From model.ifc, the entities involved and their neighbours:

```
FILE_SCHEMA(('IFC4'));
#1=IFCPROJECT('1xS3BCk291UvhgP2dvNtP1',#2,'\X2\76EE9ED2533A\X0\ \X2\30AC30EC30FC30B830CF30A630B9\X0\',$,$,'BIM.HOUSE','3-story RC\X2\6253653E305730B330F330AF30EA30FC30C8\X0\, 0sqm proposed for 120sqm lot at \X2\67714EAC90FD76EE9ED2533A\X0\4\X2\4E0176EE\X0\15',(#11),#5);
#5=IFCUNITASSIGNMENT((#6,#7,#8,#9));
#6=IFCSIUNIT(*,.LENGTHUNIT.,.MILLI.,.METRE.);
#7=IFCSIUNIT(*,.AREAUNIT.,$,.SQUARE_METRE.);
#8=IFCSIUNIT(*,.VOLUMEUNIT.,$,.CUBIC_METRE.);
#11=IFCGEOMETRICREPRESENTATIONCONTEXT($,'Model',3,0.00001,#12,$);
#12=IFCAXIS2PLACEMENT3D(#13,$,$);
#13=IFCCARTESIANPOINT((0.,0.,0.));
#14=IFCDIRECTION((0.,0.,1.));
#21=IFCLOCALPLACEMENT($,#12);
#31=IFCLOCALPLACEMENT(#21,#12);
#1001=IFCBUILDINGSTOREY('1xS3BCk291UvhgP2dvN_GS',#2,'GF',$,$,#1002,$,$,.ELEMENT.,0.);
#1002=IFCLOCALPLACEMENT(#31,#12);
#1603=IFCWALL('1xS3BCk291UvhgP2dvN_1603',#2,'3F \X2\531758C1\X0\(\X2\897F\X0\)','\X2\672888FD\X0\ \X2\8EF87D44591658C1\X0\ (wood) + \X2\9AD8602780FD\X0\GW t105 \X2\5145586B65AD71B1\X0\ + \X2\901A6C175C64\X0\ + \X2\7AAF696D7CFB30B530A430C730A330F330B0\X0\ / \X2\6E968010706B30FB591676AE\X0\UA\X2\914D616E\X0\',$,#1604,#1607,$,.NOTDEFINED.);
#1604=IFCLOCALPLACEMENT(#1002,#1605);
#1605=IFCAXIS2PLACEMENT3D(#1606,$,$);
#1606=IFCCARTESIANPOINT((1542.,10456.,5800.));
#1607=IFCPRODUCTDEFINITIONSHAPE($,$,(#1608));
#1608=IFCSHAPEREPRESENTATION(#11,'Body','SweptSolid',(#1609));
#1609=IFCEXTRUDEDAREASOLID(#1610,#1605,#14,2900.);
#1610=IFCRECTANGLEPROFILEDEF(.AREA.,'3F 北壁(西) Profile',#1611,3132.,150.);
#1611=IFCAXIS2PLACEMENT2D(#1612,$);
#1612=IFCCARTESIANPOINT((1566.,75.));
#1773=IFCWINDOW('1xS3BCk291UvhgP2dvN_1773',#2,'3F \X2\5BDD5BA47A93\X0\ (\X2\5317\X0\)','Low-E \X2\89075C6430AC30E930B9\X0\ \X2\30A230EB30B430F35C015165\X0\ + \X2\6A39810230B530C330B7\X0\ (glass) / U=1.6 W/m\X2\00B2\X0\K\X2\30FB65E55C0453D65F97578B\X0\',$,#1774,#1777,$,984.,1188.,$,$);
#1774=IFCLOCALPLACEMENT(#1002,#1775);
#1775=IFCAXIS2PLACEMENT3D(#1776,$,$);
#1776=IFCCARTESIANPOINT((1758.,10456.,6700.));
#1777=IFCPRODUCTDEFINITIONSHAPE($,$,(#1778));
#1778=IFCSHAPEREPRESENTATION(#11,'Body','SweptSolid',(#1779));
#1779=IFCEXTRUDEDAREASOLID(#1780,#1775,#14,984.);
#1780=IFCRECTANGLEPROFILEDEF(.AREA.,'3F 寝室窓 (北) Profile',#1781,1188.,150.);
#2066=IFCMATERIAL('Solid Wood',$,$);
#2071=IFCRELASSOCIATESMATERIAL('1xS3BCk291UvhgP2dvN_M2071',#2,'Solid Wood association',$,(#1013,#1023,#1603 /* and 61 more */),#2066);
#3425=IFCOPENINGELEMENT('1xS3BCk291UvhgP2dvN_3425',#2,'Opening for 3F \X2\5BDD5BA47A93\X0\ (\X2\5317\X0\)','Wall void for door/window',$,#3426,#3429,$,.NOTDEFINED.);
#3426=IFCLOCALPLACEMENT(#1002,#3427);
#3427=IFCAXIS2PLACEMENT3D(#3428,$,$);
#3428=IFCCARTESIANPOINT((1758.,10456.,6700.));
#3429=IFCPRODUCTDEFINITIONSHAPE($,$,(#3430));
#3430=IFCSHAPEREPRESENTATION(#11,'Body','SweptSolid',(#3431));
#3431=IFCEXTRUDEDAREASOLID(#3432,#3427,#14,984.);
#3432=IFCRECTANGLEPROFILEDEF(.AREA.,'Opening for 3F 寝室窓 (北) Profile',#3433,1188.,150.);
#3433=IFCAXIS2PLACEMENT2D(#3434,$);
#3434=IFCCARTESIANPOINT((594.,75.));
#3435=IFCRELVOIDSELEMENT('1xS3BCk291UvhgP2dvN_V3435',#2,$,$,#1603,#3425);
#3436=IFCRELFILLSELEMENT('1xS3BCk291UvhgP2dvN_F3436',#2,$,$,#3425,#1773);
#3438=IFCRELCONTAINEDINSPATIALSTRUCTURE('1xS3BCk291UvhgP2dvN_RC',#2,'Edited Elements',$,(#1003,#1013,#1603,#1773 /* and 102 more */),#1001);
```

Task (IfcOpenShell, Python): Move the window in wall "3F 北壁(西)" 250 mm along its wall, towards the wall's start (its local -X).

```python
import ifcopenshell
import ifcopenshell.api.geometry
import ifcopenshell.util.placement

model = ifcopenshell.open("model.ifc")

window = model.by_guid("1xS3BCk291UvhgP2dvN_1773")
opening = window.FillsVoids[0].RelatingOpeningElement
wall = opening.VoidsElements[0].RelatingBuildingElement

wall_matrix = ifcopenshell.util.placement.get_local_placement(wall.ObjectPlacement)
shift = wall_matrix[:3, 0] * -250.0
before = ifcopenshell.util.placement.get_local_placement(window.ObjectPlacement)[:3, 3].copy()

# The window is not placed relative to its opening, so move both.
for product in (opening, window):
    matrix = ifcopenshell.util.placement.get_local_placement(product.ObjectPlacement)
    matrix[:3, 3] += shift
    ifcopenshell.api.geometry.edit_object_placement(model, product=product, matrix=matrix, is_si=False)

after = ifcopenshell.util.placement.get_local_placement(window.ObjectPlacement)[:3, 3]
print("window moved by", (after - before).round(3) + 0.0)

model.write("model_rev.ifc")
```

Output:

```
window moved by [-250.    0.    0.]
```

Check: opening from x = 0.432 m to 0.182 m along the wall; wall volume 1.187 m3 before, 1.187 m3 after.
